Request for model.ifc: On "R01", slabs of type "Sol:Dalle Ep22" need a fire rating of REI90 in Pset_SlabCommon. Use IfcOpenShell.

First a look at what the model holds.

```python
import ifcopenshell
import ifcopenshell.util.element

model = ifcopenshell.open("model.ifc")
print(model.schema)
storey = next(s for s in model.by_type("IfcBuildingStorey") if s.Name == "R01")
slabs = [e for e in ifcopenshell.util.element.get_decomposition(storey) if e.is_a("IfcSlab")]
seen = {}
for e in slabs:
    element_type = ifcopenshell.util.element.get_type(e)
    key = (element_type.Name if element_type != e and element_type else None, ifcopenshell.util.element.get_pset(e, "Pset_SlabCommon", "FireRating"))
    seen[key] = seen.get(key, 0) + 1
for (name, value), count in sorted(seen.items(), key=str):
    print(count, "x", name, "|", value)
```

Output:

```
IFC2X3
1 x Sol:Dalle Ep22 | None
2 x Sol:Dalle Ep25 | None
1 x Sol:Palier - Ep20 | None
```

```python
import ifcopenshell
import ifcopenshell.api.pset
import ifcopenshell.util.element

model = ifcopenshell.open("model.ifc")

storey = next(s for s in model.by_type("IfcBuildingStorey") if s.Name == "R01")
slabs = [e for e in ifcopenshell.util.element.get_decomposition(storey) if e.is_a("IfcSlab")]

count = 0
for e in slabs:
    element_type = ifcopenshell.util.element.get_type(e)
    if element_type in (None, e) or element_type.Name != "Sol:Dalle Ep22":
        continue
    # add_pset returns the element's existing set when there is one.
    pset = ifcopenshell.api.pset.add_pset(model, product=e, name="Pset_SlabCommon")
    ifcopenshell.api.pset.edit_pset(model, pset=pset, properties={"FireRating": "REI90"})
    count += 1

print(count, "slabs updated")

model.write("model_rev.ifc")
```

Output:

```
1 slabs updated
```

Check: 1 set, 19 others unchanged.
